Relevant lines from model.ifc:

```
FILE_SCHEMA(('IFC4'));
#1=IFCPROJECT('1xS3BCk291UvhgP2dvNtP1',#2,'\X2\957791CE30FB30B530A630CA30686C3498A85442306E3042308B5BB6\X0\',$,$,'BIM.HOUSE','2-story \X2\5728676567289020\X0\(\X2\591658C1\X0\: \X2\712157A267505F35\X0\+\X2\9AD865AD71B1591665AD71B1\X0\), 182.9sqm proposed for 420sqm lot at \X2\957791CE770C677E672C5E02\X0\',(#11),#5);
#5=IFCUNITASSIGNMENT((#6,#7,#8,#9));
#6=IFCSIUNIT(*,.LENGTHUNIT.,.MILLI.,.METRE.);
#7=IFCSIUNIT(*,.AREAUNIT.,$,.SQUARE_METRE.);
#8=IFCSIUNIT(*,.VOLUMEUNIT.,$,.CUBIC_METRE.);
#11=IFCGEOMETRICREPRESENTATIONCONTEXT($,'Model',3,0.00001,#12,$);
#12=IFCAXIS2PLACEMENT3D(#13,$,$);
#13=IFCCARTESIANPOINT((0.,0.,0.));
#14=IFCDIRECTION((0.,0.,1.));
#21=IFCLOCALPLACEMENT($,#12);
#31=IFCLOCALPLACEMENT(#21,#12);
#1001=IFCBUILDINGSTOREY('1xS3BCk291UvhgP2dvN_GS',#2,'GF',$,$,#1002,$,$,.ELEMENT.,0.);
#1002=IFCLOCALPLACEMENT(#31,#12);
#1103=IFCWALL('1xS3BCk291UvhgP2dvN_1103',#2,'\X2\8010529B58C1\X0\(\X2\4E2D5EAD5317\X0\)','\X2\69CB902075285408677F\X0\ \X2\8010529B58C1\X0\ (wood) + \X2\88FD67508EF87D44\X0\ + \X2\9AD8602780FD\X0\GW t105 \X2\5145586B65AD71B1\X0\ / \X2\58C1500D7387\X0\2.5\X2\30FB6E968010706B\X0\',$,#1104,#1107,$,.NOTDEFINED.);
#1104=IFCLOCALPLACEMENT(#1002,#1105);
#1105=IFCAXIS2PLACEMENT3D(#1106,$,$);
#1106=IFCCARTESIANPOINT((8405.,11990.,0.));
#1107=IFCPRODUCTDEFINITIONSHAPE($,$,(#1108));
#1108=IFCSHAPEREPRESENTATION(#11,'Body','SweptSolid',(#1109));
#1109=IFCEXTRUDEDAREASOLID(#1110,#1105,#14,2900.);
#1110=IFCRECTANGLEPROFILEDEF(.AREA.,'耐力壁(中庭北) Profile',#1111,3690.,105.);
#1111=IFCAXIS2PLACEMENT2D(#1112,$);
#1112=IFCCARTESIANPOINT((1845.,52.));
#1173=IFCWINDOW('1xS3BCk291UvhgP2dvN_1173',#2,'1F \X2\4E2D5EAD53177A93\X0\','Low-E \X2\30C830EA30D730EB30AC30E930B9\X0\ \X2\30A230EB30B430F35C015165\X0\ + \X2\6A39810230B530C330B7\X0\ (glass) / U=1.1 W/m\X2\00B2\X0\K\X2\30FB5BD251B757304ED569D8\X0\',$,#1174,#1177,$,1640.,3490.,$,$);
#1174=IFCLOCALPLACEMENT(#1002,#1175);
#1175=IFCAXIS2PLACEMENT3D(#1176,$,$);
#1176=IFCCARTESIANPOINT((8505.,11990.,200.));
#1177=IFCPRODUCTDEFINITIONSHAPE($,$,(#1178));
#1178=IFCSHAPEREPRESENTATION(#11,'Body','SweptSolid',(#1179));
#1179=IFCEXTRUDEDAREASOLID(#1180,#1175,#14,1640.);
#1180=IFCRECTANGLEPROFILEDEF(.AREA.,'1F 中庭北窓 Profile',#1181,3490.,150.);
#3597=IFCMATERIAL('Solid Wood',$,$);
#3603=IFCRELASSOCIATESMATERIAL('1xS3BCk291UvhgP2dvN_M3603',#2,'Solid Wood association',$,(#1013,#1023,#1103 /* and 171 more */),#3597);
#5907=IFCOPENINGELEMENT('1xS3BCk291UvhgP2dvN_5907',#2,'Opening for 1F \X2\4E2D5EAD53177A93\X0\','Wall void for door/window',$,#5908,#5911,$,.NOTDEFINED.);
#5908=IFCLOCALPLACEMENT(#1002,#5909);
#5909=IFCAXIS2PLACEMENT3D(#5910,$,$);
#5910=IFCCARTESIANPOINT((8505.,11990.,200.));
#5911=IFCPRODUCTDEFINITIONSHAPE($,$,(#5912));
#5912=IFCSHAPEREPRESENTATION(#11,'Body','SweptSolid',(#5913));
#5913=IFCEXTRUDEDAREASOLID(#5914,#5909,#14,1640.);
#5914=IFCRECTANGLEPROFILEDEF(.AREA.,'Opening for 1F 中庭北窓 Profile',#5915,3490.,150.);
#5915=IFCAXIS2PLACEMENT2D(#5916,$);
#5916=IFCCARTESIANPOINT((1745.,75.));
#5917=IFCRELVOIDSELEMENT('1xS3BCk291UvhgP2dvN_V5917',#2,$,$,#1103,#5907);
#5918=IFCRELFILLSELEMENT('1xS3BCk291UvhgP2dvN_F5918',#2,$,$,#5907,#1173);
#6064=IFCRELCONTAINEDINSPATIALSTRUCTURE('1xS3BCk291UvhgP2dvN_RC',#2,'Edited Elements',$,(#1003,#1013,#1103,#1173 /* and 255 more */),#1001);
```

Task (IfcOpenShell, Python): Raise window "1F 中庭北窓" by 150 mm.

```python
import numpy as np
import ifcopenshell
import ifcopenshell.api.geometry
import ifcopenshell.util.placement
import ifcopenshell.util.unit

model = ifcopenshell.open("model.ifc")
unit_scale = ifcopenshell.util.unit.calculate_unit_scale(model)

window = model.by_guid("1xS3BCk291UvhgP2dvN_1173")
opening = window.FillsVoids[0].RelatingOpeningElement
dz = 150.0

shift = np.array([0.0, 0.0, dz])
# The window is not placed relative to its opening, so move both.
for product in (opening, window):
    matrix = ifcopenshell.util.placement.get_local_placement(product.ObjectPlacement)
    matrix[:3, 3] += shift
    ifcopenshell.api.geometry.edit_object_placement(model, product=product, matrix=matrix, is_si=False)

print(f"moved by {dz * unit_scale:+.3f} m")

model.write("model_edited.ifc")
```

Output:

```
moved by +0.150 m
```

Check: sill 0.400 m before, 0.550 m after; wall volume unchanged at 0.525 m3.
